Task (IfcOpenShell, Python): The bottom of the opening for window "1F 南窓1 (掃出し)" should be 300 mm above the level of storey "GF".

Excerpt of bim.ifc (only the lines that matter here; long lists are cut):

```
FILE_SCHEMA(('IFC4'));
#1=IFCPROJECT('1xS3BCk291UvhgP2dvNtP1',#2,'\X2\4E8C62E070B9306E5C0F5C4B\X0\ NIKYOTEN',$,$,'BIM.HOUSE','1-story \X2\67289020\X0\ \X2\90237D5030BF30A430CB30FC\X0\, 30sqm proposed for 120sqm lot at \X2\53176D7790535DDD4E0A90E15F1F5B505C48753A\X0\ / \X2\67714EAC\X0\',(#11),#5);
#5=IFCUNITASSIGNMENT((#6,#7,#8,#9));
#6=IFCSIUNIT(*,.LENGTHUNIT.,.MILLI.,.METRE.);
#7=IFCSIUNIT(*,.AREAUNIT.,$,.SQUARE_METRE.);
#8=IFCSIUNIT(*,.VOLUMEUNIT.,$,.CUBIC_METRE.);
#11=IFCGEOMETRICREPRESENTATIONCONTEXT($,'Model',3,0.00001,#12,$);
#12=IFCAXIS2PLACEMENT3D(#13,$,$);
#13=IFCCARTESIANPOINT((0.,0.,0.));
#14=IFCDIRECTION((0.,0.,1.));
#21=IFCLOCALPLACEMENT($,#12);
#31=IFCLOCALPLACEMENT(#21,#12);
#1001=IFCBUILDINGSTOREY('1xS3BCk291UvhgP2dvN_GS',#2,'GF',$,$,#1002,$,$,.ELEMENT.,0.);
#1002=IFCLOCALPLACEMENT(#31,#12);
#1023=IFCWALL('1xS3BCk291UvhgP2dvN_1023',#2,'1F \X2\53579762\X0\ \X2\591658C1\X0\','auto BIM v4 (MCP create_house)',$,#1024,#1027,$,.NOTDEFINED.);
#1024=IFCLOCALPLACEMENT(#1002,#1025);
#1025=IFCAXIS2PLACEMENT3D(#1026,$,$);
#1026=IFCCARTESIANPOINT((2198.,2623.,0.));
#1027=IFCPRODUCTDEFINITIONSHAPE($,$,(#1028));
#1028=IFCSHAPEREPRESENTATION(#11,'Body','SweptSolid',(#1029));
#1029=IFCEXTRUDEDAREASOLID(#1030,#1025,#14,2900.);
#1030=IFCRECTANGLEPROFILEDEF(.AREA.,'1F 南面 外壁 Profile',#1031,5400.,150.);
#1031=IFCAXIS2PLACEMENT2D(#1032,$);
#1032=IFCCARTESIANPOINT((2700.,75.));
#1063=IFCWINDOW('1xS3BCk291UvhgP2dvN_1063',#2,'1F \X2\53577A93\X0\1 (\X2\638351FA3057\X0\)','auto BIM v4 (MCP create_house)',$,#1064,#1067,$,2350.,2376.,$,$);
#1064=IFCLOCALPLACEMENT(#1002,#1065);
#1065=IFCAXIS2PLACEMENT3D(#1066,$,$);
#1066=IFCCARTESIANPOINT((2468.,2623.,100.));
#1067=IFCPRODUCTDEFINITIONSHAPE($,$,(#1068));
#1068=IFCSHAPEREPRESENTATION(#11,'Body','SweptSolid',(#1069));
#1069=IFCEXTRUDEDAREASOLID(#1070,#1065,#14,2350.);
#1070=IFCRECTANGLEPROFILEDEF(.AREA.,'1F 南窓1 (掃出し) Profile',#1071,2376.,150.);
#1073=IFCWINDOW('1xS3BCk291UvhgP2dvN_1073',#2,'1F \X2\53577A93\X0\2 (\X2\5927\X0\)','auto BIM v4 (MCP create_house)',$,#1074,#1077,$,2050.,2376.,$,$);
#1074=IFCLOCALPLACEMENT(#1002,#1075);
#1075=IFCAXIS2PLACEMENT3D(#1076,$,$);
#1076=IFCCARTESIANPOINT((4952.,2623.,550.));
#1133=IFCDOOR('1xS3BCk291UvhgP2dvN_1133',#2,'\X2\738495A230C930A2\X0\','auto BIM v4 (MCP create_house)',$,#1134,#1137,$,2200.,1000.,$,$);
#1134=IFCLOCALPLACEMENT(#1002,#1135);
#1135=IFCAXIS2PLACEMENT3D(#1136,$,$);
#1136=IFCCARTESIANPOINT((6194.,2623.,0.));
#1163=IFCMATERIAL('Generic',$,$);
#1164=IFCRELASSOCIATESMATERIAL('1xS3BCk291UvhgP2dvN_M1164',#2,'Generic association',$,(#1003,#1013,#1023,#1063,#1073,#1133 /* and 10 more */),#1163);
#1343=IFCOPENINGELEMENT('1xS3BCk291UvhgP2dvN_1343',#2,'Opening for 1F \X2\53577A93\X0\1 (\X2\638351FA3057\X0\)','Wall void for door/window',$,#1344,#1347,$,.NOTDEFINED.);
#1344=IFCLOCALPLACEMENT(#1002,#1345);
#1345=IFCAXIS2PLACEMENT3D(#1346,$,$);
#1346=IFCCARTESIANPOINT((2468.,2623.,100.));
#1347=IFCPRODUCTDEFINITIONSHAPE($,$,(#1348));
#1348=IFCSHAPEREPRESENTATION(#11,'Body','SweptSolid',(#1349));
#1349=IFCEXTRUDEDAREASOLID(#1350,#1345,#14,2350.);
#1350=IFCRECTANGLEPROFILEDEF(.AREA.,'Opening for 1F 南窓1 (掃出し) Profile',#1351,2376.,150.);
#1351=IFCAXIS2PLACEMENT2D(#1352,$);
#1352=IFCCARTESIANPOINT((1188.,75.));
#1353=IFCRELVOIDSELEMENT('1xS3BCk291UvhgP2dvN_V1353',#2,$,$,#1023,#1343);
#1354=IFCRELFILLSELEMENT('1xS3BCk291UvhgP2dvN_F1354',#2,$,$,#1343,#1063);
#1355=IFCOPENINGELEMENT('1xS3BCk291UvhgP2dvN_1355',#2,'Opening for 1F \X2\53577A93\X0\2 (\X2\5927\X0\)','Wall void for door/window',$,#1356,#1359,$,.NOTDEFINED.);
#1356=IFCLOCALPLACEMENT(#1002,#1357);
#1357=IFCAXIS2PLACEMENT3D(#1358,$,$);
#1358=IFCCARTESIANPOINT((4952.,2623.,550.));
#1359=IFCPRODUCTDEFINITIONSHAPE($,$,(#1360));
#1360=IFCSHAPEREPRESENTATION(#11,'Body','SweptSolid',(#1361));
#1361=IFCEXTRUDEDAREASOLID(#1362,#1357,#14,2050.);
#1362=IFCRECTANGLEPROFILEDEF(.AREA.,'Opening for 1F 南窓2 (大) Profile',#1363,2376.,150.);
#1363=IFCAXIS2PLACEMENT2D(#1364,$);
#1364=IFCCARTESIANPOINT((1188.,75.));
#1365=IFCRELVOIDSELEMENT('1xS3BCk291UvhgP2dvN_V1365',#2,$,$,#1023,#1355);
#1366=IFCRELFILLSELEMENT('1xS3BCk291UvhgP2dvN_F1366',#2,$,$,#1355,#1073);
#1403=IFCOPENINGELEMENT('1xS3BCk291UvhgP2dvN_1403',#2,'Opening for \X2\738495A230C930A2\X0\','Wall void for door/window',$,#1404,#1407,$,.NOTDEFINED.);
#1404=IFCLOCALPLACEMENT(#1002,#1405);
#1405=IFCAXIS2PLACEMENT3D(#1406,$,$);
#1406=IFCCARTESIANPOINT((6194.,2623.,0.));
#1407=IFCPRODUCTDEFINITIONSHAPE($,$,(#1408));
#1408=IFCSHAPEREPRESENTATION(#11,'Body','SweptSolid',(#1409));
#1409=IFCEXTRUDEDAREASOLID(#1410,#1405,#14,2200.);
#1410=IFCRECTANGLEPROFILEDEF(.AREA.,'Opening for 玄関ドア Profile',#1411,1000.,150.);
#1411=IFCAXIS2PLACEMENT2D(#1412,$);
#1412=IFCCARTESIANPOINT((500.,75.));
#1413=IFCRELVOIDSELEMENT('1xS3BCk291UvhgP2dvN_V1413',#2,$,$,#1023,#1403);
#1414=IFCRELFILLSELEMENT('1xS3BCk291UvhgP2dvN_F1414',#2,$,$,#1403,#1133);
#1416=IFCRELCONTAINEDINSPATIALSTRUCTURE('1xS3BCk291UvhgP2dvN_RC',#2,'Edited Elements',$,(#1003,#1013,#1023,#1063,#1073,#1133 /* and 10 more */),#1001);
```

```python
import numpy as np
import ifcopenshell
import ifcopenshell.api.geometry
import ifcopenshell.geom
import ifcopenshell.util.element
import ifcopenshell.util.placement
import ifcopenshell.util.shape
import ifcopenshell.util.unit

model = ifcopenshell.open("bim.ifc")
unit_scale = ifcopenshell.util.unit.calculate_unit_scale(model)

window = model.by_id(1063)
opening = window.FillsVoids[0].RelatingOpeningElement
storey = ifcopenshell.util.element.get_container(window, ifc_class="IfcBuildingStorey")
level = ifcopenshell.util.placement.get_local_placement(storey.ObjectPlacement)[2, 3]

# The opening's origin need not be at the sill, so measure its lowest point.
shape = ifcopenshell.geom.create_shape(ifcopenshell.geom.settings(), opening)
bottom = ifcopenshell.util.shape.get_shape_bottom_elevation(shape, shape.geometry) / unit_scale
dz = level + 300.0 - bottom

shift = np.array([0.0, 0.0, dz])
# The window is not placed relative to its opening, so move both.
for product in (opening, window):
    matrix = ifcopenshell.util.placement.get_local_placement(product.ObjectPlacement)
    matrix[:3, 3] += shift
    ifcopenshell.api.geometry.edit_object_placement(model, product=product, matrix=matrix, is_si=False)

print(f"moved by {dz * unit_scale:+.3f} m")

model.write("bim_rev.ifc")
```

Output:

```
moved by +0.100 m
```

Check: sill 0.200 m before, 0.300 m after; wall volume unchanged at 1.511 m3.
